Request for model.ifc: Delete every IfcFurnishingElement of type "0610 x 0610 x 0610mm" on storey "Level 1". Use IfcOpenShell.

First a look at what the model holds.

```python
import ifcopenshell
import ifcopenshell.util.element

model = ifcopenshell.open("model.ifc")
print(model.schema)
storey = next(s for s in model.by_type("IfcBuildingStorey") if s.Name == "Level 1")
furniture = [e for e in ifcopenshell.util.element.get_decomposition(storey) if e.is_a("IfcFurnishingElement")]
seen = {}
for e in furniture:
    element_type = ifcopenshell.util.element.get_type(e)
    name = element_type.Name if element_type not in (None, e) else None
    seen[name] = seen.get(name, 0) + 1
for name, count in sorted(seen.items(), key=str):
    print(count, "x", name)
```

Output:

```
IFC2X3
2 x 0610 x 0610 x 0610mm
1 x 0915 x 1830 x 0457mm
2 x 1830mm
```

```python
import ifcopenshell
import ifcopenshell.api.root
import ifcopenshell.util.element

model = ifcopenshell.open("model.ifc")

storey = next(s for s in model.by_type("IfcBuildingStorey") if s.Name == "Level 1")
furniture = [e for e in ifcopenshell.util.element.get_decomposition(storey) if e.is_a("IfcFurnishingElement")]
targets = [e for e in furniture if (t := ifcopenshell.util.element.get_type(e)) not in (None, e) and t.Name == "0610 x 0610 x 0610mm"]

for e in targets:
    ifcopenshell.api.root.remove_product(model, product=e)
print(len(targets), "removed")

model.write("model_v2.ifc")
```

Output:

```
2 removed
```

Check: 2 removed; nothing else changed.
